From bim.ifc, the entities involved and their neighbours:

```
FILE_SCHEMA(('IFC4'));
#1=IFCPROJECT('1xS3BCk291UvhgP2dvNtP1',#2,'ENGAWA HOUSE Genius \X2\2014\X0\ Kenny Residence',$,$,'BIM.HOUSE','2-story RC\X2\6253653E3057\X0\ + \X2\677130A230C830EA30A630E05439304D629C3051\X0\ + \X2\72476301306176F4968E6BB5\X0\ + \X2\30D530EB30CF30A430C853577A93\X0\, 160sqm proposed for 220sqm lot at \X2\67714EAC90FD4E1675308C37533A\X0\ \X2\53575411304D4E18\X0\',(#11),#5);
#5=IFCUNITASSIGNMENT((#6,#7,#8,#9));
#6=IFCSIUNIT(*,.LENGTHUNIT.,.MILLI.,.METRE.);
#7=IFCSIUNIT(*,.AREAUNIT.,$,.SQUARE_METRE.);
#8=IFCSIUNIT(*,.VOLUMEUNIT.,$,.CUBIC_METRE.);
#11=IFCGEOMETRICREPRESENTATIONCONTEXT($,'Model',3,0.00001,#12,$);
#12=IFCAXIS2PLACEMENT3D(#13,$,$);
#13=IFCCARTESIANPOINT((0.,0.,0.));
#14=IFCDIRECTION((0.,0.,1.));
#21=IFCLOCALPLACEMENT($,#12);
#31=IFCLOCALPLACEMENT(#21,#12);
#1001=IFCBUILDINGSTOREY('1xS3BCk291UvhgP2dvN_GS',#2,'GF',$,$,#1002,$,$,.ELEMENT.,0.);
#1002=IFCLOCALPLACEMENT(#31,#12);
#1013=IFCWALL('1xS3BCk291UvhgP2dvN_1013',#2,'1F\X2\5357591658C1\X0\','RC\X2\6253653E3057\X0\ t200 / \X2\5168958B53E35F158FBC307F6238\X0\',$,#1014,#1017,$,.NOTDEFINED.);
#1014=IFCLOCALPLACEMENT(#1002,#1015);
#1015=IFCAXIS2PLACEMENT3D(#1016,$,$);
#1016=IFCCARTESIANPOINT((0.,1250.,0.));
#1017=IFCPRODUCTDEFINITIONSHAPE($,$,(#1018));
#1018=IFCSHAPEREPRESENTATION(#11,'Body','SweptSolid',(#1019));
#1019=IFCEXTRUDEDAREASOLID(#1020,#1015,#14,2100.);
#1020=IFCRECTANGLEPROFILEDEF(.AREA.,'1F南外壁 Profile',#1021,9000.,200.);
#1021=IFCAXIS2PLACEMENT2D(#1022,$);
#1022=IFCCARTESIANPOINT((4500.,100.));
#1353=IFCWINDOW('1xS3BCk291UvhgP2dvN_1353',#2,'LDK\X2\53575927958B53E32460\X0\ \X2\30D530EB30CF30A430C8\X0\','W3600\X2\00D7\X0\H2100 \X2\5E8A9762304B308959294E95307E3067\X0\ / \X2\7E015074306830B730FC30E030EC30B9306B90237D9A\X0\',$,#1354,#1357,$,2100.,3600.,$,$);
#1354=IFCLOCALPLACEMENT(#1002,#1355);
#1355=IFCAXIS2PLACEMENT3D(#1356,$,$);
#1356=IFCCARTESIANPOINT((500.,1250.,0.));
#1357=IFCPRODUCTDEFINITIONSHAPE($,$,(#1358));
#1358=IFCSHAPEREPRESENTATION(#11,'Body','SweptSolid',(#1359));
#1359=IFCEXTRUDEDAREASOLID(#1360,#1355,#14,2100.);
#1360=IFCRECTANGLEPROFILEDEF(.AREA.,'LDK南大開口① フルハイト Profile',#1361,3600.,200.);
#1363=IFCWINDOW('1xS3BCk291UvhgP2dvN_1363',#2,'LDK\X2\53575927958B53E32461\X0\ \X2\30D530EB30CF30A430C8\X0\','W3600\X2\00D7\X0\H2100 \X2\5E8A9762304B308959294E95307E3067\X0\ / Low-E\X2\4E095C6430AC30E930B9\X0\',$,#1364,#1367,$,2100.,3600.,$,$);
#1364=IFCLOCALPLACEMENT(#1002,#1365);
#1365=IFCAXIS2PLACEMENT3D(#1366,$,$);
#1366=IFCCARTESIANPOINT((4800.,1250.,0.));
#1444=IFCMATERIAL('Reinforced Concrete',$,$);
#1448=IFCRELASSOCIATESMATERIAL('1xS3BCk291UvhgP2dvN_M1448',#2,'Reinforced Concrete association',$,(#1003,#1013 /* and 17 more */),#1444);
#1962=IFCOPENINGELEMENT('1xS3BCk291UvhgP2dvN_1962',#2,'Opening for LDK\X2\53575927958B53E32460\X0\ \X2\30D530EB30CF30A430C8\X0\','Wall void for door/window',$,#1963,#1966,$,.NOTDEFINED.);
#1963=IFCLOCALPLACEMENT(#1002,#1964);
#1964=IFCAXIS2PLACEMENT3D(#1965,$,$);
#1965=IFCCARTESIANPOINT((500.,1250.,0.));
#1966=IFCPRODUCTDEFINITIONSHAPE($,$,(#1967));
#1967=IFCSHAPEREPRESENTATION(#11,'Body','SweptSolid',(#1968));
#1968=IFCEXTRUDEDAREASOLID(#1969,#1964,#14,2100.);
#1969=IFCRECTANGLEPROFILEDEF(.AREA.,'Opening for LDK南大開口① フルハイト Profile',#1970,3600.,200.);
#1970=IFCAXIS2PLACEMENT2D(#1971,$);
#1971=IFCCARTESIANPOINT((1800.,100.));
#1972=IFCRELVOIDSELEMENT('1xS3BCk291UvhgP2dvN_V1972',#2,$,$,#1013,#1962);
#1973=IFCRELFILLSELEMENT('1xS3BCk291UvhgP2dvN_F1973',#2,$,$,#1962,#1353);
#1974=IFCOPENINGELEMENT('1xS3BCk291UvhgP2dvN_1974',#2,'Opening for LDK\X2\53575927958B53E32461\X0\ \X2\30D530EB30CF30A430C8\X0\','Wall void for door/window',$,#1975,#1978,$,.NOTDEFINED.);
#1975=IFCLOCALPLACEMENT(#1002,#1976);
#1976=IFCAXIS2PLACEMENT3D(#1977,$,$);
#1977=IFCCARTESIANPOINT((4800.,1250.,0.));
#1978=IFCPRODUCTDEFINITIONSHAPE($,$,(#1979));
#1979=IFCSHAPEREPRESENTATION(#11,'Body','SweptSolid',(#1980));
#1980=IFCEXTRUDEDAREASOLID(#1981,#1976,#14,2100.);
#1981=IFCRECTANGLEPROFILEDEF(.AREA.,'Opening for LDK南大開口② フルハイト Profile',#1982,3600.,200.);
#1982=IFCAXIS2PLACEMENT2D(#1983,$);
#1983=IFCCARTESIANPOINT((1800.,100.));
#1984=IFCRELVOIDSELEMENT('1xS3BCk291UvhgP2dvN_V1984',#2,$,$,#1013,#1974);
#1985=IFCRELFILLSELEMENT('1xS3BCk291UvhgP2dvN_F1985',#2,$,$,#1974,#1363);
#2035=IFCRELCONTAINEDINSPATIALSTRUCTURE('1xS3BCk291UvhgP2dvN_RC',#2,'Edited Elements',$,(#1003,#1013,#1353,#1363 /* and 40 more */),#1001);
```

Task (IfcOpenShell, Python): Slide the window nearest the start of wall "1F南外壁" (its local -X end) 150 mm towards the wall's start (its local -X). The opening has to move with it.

```python
import ifcopenshell
import ifcopenshell.api.geometry
import ifcopenshell.util.placement
import ifcopenshell.util.unit

model = ifcopenshell.open("bim.ifc")
unit_scale = ifcopenshell.util.unit.calculate_unit_scale(model)

window = model.by_guid("1xS3BCk291UvhgP2dvN_1353")
opening = window.FillsVoids[0].RelatingOpeningElement
wall = opening.VoidsElements[0].RelatingBuildingElement

wall_matrix = ifcopenshell.util.placement.get_local_placement(wall.ObjectPlacement)
shift = wall_matrix[:3, 0] * -0.15 / unit_scale
before = ifcopenshell.util.placement.get_local_placement(window.ObjectPlacement)[:3, 3].copy()

# The window is not placed relative to its opening, so move both.
for product in (opening, window):
    matrix = ifcopenshell.util.placement.get_local_placement(product.ObjectPlacement)
    matrix[:3, 3] += shift
    ifcopenshell.api.geometry.edit_object_placement(model, product=product, matrix=matrix, is_si=False)

after = ifcopenshell.util.placement.get_local_placement(window.ObjectPlacement)[:3, 3]
print("window moved by", (after - before).round(3) + 0.0)

model.write("bim-out.ifc")
```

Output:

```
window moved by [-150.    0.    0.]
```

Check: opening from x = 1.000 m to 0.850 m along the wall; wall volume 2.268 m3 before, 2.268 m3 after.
